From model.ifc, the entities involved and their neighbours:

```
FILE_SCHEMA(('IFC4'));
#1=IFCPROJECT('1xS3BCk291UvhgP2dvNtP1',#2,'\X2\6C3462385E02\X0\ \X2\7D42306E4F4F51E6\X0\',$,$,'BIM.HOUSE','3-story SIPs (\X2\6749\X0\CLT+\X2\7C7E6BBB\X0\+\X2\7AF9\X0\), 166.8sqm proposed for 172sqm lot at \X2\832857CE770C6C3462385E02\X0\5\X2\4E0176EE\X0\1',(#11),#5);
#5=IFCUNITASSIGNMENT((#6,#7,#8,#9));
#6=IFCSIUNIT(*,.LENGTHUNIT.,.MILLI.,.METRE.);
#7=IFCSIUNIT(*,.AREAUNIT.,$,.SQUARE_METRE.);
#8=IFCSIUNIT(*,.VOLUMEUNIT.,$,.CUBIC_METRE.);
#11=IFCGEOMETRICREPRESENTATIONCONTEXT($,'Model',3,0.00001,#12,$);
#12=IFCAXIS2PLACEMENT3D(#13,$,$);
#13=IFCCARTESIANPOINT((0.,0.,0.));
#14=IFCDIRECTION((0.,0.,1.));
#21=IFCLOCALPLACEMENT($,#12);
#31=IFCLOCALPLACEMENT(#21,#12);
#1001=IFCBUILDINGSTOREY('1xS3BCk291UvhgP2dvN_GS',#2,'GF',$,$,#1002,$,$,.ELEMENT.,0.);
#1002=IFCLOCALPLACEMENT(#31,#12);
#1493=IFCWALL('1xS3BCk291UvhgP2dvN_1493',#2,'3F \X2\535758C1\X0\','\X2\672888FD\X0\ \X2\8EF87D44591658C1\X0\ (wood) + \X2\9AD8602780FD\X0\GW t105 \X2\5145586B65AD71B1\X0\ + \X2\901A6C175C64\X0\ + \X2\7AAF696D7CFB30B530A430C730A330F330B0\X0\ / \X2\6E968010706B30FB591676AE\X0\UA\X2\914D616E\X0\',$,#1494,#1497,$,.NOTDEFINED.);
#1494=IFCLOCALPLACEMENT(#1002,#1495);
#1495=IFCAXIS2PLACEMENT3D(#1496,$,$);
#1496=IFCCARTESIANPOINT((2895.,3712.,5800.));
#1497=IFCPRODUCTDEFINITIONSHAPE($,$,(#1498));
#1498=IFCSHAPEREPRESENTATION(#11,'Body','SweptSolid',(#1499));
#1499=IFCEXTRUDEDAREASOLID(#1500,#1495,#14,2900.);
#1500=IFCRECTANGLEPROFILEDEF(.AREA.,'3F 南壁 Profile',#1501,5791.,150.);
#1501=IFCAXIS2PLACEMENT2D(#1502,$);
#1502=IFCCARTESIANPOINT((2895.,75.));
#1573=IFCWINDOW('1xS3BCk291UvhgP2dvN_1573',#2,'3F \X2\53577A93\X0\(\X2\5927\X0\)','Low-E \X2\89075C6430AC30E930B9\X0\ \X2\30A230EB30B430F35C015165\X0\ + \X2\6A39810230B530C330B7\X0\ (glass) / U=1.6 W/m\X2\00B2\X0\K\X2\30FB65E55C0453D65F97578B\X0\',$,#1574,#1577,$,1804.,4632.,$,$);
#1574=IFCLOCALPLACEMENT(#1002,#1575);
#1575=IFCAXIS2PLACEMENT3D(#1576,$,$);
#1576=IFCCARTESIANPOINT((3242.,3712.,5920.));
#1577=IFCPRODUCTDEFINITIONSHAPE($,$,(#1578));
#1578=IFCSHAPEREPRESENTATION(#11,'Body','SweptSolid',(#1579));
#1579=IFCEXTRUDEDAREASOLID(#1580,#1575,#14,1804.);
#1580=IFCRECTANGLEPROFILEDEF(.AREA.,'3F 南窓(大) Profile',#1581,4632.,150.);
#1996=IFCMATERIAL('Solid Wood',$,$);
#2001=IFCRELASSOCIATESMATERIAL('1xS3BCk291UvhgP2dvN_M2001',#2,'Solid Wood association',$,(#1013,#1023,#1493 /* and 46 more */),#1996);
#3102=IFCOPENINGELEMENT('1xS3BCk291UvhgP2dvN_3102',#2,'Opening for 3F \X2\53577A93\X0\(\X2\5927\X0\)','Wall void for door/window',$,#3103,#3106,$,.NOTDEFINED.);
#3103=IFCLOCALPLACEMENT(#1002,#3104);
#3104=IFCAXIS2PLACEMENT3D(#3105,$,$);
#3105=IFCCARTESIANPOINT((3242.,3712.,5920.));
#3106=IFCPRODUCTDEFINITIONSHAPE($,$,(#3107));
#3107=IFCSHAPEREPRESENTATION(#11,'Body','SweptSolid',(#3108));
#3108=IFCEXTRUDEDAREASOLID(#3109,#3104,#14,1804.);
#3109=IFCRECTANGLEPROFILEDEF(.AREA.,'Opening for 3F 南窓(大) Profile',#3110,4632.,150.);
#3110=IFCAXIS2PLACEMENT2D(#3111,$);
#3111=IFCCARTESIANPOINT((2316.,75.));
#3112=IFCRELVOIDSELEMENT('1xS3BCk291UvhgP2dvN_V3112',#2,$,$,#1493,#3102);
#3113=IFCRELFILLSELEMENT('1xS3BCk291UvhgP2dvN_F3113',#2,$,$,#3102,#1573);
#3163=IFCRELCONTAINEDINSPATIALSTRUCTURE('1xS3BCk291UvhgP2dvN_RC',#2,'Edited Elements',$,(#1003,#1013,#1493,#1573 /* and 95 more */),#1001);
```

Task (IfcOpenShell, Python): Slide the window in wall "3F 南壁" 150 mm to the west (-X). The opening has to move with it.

```python
import ifcopenshell
import ifcopenshell.api.geometry
import ifcopenshell.util.placement

model = ifcopenshell.open("model.ifc")

window = model.by_id(1573)
opening = window.FillsVoids[0].RelatingOpeningElement
wall = opening.VoidsElements[0].RelatingBuildingElement

wall_matrix = ifcopenshell.util.placement.get_local_placement(wall.ObjectPlacement)
shift = wall_matrix[:3, 0] * -150.0
before = ifcopenshell.util.placement.get_local_placement(window.ObjectPlacement)[:3, 3].copy()

# The window is not placed relative to its opening, so move both.
for product in (opening, window):
    matrix = ifcopenshell.util.placement.get_local_placement(product.ObjectPlacement)
    matrix[:3, 3] += shift
    ifcopenshell.api.geometry.edit_object_placement(model, product=product, matrix=matrix, is_si=False)

after = ifcopenshell.util.placement.get_local_placement(window.ObjectPlacement)[:3, 3]
print("window moved by", (after - before).round(3) + 0.0)

model.write("model_rev.ifc")
```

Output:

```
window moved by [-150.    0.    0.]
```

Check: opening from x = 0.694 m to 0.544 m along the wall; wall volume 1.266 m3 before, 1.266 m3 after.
